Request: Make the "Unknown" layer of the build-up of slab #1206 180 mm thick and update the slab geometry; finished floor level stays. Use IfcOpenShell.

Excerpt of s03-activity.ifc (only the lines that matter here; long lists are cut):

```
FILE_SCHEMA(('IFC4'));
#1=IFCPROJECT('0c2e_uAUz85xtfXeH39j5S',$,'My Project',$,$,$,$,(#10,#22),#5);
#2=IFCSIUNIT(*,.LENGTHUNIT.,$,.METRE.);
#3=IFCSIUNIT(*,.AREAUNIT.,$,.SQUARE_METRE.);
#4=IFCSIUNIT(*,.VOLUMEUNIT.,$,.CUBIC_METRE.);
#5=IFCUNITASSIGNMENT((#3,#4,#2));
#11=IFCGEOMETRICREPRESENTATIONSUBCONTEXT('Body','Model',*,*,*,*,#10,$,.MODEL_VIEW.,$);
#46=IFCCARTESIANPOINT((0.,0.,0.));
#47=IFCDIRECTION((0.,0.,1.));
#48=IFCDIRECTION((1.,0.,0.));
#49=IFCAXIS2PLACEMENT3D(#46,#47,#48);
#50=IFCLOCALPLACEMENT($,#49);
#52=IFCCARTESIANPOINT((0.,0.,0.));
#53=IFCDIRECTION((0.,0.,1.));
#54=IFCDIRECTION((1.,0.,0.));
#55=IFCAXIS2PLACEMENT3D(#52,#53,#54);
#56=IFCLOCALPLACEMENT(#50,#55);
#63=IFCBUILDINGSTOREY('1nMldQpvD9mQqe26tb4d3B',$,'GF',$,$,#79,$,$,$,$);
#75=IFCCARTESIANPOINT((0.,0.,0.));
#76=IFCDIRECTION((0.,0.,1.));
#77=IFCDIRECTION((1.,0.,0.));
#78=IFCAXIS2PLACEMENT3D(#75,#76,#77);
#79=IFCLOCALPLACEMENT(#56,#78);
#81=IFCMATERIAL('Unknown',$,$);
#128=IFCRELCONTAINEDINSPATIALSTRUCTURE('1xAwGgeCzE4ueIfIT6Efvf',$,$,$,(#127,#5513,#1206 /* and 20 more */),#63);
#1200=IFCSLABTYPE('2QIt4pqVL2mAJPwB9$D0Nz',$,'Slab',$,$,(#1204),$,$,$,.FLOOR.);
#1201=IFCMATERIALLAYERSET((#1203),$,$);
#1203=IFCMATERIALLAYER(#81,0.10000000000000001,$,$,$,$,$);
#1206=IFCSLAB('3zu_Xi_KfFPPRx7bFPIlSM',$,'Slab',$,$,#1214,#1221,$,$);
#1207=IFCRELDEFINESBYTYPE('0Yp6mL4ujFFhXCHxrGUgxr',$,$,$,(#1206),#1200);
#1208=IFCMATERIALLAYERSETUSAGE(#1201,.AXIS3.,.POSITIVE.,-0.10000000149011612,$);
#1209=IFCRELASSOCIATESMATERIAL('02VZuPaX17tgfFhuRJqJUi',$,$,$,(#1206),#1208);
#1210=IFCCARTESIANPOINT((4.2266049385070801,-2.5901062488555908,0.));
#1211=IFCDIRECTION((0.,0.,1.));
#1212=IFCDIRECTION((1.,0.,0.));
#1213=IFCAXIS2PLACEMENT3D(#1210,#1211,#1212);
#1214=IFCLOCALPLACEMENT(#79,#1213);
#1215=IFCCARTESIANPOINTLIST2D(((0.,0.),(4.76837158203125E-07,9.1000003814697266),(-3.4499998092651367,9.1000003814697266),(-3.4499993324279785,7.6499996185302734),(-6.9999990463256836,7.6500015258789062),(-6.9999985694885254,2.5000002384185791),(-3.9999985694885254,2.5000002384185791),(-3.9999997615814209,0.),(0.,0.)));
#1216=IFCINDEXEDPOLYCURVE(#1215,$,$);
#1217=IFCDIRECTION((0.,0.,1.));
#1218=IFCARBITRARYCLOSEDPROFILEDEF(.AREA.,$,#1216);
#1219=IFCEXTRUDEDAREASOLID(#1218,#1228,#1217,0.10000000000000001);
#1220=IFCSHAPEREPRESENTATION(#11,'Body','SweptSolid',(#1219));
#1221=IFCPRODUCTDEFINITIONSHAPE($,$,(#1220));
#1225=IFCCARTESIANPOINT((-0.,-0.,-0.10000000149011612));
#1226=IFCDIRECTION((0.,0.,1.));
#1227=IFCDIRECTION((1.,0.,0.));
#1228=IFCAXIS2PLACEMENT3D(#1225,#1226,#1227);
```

```python
import ifcopenshell
import ifcopenshell.util.element
import ifcopenshell.util.representation
import ifcopenshell.util.unit

model = ifcopenshell.open("s03-activity.ifc")
unit_scale = ifcopenshell.util.unit.calculate_unit_scale(model)

layer_set = model.by_id(1201)
layer = next(l for l in layer_set.MaterialLayers if l.Material and l.Material.Name == "Unknown")
change = 0.18 / unit_scale - layer.LayerThickness
layer.LayerThickness += change

# Geometry does not follow the layer set by itself.
slabs = [e for e in ifcopenshell.util.element.get_elements_by_material(model, layer_set) if e.is_a("IfcSlab")]
for slab in sorted(slabs, key=lambda e: e.id()):
    body = ifcopenshell.util.representation.get_representation(slab, "Model", "Body")
    solid = body.Items[0]
    old_depth = solid.Depth
    solid.Depth += change
    # Extruded upwards: lower the start of the extrusion so the top stays.
    x, y, z = solid.Position.Location.Coordinates
    solid.Position.Location = model.createIfcCartesianPoint((x, y, z - change))
    print(slab.id(), f"{old_depth:g} -> {solid.Depth:g}")

# The layers are counted up from the underside, which has moved.
for usage in {ifcopenshell.util.element.get_material(slab) for slab in slabs}:
    usage.OffsetFromReferenceLine -= change

model.write("s03-activity_edited.ifc")
```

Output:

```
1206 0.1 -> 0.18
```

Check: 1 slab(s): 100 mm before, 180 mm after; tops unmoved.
